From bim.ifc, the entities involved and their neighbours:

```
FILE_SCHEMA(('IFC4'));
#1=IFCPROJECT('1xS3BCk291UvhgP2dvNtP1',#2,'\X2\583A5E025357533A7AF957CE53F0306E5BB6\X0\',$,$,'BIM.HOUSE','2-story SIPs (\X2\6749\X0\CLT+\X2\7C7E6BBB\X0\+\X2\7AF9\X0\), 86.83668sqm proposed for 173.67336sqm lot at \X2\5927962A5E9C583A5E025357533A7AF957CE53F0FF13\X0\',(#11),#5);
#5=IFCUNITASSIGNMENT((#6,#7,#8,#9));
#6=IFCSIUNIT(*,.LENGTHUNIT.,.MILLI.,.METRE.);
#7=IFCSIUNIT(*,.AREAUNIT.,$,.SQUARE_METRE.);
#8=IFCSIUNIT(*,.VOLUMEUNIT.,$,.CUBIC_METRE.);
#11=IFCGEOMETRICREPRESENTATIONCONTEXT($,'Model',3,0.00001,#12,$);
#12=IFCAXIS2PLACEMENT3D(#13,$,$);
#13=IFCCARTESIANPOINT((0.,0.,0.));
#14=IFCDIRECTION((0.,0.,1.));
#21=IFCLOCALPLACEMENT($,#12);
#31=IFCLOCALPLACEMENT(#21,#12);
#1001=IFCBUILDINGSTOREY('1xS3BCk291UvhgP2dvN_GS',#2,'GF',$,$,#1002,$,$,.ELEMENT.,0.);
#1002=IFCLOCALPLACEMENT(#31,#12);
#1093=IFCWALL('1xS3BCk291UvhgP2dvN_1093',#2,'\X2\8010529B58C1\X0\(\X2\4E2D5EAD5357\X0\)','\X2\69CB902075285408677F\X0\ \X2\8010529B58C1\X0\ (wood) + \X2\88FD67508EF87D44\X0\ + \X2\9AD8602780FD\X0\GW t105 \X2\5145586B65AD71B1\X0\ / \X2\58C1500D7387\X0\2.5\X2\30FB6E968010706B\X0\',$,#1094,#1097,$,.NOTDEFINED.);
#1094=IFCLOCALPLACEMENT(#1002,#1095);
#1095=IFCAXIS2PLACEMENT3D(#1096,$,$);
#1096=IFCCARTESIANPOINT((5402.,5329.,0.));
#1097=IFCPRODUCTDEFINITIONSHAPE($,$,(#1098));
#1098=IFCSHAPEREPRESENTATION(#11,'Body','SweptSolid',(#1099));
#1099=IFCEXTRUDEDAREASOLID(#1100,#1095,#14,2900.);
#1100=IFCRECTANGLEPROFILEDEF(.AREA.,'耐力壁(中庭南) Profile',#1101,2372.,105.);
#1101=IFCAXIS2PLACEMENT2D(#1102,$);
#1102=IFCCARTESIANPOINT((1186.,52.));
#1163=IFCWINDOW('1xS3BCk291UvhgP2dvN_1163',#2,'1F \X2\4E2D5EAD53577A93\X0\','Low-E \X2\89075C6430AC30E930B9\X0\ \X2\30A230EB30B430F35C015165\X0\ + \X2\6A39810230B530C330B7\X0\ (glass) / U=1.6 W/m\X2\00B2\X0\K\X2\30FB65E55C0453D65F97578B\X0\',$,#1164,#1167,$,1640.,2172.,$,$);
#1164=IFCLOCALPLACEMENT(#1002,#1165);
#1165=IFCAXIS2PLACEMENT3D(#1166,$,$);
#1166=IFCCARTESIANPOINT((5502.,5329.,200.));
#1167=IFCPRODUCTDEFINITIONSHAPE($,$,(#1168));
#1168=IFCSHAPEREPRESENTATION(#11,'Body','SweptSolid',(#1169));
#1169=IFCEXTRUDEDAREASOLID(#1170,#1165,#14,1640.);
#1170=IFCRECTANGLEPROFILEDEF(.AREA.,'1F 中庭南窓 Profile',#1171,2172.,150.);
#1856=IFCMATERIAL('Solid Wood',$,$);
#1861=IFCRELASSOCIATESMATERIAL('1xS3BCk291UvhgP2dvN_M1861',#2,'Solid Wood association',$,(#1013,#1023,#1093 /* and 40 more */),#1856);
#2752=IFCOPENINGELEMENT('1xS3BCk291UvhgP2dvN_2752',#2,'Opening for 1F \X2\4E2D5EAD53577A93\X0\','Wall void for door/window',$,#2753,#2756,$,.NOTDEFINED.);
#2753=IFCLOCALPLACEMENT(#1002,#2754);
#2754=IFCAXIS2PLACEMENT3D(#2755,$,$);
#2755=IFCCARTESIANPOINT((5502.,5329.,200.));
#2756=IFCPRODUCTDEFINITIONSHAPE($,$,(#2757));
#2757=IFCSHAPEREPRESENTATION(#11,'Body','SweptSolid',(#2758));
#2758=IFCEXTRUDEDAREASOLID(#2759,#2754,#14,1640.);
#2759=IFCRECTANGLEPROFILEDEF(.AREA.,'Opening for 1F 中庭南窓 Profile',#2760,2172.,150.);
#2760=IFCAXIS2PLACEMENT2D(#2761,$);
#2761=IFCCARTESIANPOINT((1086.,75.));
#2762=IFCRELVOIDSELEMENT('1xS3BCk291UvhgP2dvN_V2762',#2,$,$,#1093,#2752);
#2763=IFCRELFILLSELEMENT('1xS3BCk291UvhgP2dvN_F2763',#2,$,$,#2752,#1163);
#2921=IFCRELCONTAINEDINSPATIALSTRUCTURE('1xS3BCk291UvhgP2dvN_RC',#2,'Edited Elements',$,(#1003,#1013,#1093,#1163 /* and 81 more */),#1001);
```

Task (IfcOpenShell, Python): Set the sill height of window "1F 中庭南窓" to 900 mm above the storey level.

```python
import numpy as np
import ifcopenshell
import ifcopenshell.api.geometry
import ifcopenshell.geom
import ifcopenshell.util.element
import ifcopenshell.util.placement
import ifcopenshell.util.shape
import ifcopenshell.util.unit

model = ifcopenshell.open("bim.ifc")
unit_scale = ifcopenshell.util.unit.calculate_unit_scale(model)

window = model.by_guid("1xS3BCk291UvhgP2dvN_1163")
opening = window.FillsVoids[0].RelatingOpeningElement
storey = ifcopenshell.util.element.get_container(window, ifc_class="IfcBuildingStorey")
level = ifcopenshell.util.placement.get_local_placement(storey.ObjectPlacement)[2, 3]

# The opening's origin need not be at the sill, so measure its lowest point.
shape = ifcopenshell.geom.create_shape(ifcopenshell.geom.settings(), opening)
bottom = ifcopenshell.util.shape.get_shape_bottom_elevation(shape, shape.geometry) / unit_scale
dz = level + 0.9 / unit_scale - bottom

shift = np.array([0.0, 0.0, dz])
# The window is not placed relative to its opening, so move both.
for product in (opening, window):
    matrix = ifcopenshell.util.placement.get_local_placement(product.ObjectPlacement)
    matrix[:3, 3] += shift
    ifcopenshell.api.geometry.edit_object_placement(model, product=product, matrix=matrix, is_si=False)

print(f"moved by {dz * unit_scale:+.3f} m")

model.write("bim_edited.ifc")
```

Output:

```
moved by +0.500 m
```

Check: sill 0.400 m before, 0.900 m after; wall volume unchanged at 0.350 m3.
